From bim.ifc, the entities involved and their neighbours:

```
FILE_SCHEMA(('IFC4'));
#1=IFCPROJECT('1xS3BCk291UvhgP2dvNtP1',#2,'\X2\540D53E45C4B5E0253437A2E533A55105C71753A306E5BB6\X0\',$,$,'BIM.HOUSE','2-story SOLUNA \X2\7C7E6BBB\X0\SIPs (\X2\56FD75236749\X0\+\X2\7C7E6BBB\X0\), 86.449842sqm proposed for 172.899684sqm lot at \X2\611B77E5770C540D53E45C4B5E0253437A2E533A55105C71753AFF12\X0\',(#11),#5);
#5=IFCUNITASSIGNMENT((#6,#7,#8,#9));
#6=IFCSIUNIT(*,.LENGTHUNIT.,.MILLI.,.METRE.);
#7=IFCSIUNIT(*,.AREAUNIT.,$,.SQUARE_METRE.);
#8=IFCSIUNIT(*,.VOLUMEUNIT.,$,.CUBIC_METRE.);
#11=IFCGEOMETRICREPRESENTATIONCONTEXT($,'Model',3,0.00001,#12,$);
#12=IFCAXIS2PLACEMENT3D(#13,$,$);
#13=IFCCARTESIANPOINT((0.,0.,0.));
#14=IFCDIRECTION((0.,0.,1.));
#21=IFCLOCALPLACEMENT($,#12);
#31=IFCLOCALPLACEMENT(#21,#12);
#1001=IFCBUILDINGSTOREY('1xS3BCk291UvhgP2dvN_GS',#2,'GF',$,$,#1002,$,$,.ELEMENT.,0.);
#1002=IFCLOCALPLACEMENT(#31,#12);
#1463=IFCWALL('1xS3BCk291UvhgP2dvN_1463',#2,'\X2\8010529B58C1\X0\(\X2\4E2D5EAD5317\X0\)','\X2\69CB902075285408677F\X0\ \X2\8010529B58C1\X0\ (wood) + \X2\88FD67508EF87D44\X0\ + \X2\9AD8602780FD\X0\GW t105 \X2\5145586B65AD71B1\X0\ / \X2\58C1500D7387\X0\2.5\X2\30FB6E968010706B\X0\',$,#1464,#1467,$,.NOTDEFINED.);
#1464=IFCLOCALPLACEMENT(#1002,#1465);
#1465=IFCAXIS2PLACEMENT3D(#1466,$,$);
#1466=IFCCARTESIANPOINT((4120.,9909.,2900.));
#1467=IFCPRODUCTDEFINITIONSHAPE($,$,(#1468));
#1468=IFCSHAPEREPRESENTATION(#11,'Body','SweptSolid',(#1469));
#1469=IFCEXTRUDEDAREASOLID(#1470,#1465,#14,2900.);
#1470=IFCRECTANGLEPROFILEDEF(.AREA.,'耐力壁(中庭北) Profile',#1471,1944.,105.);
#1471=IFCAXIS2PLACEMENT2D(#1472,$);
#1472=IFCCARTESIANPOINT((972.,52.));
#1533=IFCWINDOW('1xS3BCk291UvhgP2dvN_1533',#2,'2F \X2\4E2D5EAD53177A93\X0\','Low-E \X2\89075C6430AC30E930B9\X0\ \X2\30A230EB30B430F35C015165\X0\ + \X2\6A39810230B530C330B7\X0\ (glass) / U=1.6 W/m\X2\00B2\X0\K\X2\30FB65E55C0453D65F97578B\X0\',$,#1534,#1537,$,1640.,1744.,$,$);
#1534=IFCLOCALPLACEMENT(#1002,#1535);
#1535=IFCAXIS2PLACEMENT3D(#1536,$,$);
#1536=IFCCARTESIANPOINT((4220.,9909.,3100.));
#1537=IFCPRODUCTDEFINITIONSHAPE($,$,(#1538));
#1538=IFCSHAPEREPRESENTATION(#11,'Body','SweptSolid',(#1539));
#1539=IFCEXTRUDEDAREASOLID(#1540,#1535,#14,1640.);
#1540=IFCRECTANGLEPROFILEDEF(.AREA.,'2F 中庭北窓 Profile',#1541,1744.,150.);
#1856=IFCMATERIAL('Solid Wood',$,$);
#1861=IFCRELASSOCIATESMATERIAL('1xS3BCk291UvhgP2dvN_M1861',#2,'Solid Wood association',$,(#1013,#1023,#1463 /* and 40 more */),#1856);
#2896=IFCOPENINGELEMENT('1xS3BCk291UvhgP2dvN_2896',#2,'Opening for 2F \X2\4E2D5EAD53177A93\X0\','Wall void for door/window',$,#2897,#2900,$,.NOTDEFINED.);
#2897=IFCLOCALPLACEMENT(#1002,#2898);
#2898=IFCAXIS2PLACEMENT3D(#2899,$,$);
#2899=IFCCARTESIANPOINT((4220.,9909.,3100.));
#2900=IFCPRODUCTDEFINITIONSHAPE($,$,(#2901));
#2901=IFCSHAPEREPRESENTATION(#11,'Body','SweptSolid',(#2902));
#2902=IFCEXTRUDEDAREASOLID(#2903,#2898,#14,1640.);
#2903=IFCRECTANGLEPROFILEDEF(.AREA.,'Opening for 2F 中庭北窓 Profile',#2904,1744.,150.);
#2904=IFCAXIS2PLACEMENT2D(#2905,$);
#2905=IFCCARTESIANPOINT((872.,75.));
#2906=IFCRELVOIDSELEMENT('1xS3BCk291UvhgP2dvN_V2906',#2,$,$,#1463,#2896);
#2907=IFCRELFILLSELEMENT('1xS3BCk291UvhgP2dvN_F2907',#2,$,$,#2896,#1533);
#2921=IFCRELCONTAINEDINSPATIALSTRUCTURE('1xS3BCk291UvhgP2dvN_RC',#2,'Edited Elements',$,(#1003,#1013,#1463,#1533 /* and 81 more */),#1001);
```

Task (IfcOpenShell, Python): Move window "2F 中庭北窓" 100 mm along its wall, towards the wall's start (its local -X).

```python
import ifcopenshell
import ifcopenshell.api.geometry
import ifcopenshell.util.placement
import ifcopenshell.util.unit

model = ifcopenshell.open("bim.ifc")
unit_scale = ifcopenshell.util.unit.calculate_unit_scale(model)

window = model.by_guid("1xS3BCk291UvhgP2dvN_1533")
opening = window.FillsVoids[0].RelatingOpeningElement
wall = opening.VoidsElements[0].RelatingBuildingElement

wall_matrix = ifcopenshell.util.placement.get_local_placement(wall.ObjectPlacement)
shift = wall_matrix[:3, 0] * -0.1 / unit_scale
before = ifcopenshell.util.placement.get_local_placement(window.ObjectPlacement)[:3, 3].copy()

# The window is not placed relative to its opening, so move both.
for product in (opening, window):
    matrix = ifcopenshell.util.placement.get_local_placement(product.ObjectPlacement)
    matrix[:3, 3] += shift
    ifcopenshell.api.geometry.edit_object_placement(model, product=product, matrix=matrix, is_si=False)

after = ifcopenshell.util.placement.get_local_placement(window.ObjectPlacement)[:3, 3]
print("window moved by", (after - before).round(3) + 0.0)

model.write("bim-out.ifc")
```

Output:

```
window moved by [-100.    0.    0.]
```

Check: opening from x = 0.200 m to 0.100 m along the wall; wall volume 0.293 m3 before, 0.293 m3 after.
